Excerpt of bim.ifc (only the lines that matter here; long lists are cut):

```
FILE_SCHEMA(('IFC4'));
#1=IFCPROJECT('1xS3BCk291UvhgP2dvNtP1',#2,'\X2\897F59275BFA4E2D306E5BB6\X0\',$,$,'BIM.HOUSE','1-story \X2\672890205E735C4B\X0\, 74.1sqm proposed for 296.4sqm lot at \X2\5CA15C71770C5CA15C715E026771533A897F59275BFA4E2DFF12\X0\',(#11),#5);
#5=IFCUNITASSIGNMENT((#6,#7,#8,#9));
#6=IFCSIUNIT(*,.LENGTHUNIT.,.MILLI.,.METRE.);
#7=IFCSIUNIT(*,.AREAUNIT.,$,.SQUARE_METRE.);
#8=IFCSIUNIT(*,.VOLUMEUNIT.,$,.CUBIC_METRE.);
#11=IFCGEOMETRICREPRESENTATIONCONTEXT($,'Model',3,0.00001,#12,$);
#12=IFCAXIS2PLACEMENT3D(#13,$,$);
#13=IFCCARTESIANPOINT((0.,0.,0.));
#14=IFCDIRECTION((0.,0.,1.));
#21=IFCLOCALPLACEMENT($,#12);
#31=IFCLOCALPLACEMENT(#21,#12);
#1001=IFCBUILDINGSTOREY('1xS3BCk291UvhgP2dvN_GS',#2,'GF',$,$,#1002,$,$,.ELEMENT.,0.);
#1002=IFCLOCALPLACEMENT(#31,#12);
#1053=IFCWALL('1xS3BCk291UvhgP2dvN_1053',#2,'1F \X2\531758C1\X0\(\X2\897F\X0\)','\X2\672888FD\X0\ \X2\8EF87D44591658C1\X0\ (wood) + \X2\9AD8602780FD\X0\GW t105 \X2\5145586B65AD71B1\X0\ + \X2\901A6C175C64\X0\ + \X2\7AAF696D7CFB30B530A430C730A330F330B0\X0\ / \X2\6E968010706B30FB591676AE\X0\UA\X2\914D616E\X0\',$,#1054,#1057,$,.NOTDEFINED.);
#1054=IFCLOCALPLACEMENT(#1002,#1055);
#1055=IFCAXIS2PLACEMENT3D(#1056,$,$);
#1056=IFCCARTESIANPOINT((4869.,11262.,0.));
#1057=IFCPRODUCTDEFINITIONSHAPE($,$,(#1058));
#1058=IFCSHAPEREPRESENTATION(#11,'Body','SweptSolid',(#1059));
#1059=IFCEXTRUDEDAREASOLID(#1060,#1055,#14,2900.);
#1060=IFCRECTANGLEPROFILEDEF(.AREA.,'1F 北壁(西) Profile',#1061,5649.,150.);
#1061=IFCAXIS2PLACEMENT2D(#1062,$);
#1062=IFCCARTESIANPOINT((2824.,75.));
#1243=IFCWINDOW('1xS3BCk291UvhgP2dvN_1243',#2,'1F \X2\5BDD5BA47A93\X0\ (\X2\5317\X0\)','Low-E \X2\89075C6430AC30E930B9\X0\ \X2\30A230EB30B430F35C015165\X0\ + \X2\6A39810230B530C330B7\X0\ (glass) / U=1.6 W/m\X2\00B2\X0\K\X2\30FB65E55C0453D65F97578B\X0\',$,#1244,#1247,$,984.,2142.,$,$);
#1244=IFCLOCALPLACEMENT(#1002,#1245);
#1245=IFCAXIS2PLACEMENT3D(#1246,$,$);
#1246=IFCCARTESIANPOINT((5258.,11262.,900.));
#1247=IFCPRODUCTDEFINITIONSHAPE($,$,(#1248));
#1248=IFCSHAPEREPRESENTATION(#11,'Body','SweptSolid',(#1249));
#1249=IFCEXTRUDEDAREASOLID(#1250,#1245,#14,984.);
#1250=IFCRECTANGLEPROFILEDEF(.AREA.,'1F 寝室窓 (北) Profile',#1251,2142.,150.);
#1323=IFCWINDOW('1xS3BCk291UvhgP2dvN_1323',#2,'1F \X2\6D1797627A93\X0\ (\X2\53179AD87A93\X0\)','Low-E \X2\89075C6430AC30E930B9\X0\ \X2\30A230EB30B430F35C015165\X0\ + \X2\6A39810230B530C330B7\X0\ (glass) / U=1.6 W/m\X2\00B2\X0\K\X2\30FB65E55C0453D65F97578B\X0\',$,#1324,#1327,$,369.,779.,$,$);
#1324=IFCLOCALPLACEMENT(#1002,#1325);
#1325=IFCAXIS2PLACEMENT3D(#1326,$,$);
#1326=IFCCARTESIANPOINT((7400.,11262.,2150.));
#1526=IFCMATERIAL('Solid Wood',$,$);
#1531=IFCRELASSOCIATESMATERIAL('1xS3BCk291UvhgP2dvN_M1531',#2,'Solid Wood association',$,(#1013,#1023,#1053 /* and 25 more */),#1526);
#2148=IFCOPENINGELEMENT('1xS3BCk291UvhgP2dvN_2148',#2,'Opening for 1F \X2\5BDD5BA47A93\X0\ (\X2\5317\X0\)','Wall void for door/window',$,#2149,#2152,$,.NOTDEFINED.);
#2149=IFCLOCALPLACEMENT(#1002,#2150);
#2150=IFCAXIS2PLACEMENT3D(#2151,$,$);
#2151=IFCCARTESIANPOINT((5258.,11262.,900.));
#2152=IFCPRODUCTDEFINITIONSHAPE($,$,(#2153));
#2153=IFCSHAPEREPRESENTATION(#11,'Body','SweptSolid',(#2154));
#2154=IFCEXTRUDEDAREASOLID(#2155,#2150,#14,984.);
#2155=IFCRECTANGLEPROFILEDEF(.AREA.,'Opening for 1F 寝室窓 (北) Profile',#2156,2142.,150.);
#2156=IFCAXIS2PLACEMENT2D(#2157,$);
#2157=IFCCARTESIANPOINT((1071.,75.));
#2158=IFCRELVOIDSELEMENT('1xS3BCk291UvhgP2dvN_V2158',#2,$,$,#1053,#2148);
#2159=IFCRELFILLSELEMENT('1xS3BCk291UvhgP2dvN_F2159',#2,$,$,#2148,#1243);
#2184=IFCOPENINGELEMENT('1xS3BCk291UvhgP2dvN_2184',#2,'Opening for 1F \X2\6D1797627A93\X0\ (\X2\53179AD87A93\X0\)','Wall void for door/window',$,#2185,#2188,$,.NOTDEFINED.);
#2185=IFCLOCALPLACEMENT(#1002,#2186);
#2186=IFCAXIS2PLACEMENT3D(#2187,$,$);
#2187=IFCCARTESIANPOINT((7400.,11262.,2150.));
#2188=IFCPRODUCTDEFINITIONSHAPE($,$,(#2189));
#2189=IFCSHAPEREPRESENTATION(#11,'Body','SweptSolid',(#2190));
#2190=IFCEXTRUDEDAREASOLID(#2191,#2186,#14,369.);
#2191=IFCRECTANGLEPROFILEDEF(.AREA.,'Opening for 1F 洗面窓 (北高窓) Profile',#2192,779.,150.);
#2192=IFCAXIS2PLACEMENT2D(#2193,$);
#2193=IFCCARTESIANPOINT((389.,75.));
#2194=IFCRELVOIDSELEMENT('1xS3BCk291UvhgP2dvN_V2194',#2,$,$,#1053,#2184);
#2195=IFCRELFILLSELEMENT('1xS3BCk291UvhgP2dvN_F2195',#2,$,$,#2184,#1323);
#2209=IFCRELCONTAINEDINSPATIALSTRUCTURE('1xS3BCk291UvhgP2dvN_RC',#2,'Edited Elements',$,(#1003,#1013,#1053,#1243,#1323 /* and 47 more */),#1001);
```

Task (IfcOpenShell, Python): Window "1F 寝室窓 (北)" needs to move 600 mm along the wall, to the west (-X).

```python
import ifcopenshell
import ifcopenshell.api.geometry
import ifcopenshell.util.placement
import ifcopenshell.util.unit

model = ifcopenshell.open("bim.ifc")
unit_scale = ifcopenshell.util.unit.calculate_unit_scale(model)

window = model.by_guid("1xS3BCk291UvhgP2dvN_1243")
opening = window.FillsVoids[0].RelatingOpeningElement
wall = opening.VoidsElements[0].RelatingBuildingElement

wall_matrix = ifcopenshell.util.placement.get_local_placement(wall.ObjectPlacement)
shift = wall_matrix[:3, 0] * -0.6 / unit_scale
before = ifcopenshell.util.placement.get_local_placement(window.ObjectPlacement)[:3, 3].copy()

# The window is not placed relative to its opening, so move both.
for product in (opening, window):
    matrix = ifcopenshell.util.placement.get_local_placement(product.ObjectPlacement)
    matrix[:3, 3] += shift
    ifcopenshell.api.geometry.edit_object_placement(model, product=product, matrix=matrix, is_si=False)

after = ifcopenshell.util.placement.get_local_placement(window.ObjectPlacement)[:3, 3]
print("window moved by", (after - before).round(3) + 0.0)

model.write("bim_rev.ifc")
```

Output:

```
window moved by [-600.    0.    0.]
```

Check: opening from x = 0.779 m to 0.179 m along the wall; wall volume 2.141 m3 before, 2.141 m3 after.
